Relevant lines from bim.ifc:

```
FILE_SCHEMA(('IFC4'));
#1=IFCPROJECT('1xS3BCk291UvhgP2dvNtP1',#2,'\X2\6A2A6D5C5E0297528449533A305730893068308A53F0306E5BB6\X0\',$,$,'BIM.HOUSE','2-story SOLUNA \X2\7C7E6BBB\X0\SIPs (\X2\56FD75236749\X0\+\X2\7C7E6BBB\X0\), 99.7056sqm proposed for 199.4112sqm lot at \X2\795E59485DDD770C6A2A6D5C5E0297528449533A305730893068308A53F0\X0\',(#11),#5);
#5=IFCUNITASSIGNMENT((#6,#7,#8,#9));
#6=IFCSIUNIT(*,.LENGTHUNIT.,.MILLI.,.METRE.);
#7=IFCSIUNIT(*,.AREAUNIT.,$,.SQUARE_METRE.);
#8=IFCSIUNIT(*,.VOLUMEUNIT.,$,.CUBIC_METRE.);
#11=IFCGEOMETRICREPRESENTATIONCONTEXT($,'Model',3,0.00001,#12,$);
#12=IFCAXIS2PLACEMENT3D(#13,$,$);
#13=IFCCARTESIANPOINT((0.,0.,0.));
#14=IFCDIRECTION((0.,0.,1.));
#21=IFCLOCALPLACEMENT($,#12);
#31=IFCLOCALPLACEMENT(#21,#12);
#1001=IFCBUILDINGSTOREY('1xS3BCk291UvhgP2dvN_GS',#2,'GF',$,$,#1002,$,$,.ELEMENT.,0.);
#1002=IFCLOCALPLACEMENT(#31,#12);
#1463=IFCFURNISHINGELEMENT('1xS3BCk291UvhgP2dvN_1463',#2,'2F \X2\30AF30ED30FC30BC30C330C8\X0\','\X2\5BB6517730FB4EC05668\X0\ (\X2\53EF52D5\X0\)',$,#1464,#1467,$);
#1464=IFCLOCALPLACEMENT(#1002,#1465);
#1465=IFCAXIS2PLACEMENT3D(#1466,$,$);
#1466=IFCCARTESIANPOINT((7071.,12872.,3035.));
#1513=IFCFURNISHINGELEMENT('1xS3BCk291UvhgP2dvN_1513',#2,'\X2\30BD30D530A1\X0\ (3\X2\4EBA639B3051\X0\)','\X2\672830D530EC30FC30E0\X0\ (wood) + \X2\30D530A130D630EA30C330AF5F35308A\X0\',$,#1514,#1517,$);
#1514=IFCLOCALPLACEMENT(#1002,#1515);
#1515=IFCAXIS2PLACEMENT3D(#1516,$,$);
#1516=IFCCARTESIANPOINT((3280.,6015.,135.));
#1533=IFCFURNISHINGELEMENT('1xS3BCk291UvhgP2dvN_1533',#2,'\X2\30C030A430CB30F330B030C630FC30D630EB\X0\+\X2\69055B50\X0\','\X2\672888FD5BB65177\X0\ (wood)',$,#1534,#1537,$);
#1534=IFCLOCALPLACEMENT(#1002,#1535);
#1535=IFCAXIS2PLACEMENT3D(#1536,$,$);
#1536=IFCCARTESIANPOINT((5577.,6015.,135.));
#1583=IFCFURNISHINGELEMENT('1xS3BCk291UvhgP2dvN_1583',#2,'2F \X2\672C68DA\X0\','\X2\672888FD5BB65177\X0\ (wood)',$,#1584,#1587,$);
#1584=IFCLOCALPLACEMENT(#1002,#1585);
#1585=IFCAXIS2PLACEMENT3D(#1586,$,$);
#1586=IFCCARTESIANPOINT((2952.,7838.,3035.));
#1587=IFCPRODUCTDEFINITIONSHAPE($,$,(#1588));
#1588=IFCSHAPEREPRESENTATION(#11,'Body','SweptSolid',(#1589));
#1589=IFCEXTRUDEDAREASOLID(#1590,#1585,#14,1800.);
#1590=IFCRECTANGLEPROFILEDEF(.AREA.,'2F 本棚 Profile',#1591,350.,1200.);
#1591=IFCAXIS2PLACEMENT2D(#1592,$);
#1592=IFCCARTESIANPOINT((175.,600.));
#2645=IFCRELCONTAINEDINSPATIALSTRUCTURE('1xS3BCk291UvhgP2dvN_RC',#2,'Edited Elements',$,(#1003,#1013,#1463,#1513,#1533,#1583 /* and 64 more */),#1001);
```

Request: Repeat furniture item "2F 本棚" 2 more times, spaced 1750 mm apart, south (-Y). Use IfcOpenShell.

```python
import numpy as np
import ifcopenshell
import ifcopenshell.api.geometry
import ifcopenshell.api.root
import ifcopenshell.util.element
import ifcopenshell.util.placement

model = ifcopenshell.open("bim.ifc")


def reuse_history(source, copy):
    """copy_class also copies each property set's owner history, people and application; keep the originals."""
    for rel in copy.IsDefinedBy:
        if rel.is_a("IfcRelDefinesByProperties") and (history := rel.RelatingPropertyDefinition.OwnerHistory):
            rel.RelatingPropertyDefinition.OwnerHistory = source.OwnerHistory
            ifcopenshell.util.element.remove_deep2(model, history)


source = model.by_guid("1xS3BCk291UvhgP2dvN_1583")
base = ifcopenshell.util.placement.get_local_placement(source.ObjectPlacement)
step = np.array([0.0, -1.0, 0.0]) * 1750.0

for i in range(1, 3):
    copy = ifcopenshell.api.root.copy_class(model, product=source)
    copy.Representation = ifcopenshell.util.element.copy_deep(
        model, source.Representation, exclude=["IfcGeometricRepresentationContext", "IfcRepresentationMap"]
    )
    reuse_history(source, copy)
    matrix = base.copy()
    matrix[:3, 3] += i * step
    print("added at", matrix[:3, 3].round(3) + 0.0)
    ifcopenshell.api.geometry.edit_object_placement(model, product=copy, matrix=matrix, is_si=False)

model.write("bim_rev.ifc")
```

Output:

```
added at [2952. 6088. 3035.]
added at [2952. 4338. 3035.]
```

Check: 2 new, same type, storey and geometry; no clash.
